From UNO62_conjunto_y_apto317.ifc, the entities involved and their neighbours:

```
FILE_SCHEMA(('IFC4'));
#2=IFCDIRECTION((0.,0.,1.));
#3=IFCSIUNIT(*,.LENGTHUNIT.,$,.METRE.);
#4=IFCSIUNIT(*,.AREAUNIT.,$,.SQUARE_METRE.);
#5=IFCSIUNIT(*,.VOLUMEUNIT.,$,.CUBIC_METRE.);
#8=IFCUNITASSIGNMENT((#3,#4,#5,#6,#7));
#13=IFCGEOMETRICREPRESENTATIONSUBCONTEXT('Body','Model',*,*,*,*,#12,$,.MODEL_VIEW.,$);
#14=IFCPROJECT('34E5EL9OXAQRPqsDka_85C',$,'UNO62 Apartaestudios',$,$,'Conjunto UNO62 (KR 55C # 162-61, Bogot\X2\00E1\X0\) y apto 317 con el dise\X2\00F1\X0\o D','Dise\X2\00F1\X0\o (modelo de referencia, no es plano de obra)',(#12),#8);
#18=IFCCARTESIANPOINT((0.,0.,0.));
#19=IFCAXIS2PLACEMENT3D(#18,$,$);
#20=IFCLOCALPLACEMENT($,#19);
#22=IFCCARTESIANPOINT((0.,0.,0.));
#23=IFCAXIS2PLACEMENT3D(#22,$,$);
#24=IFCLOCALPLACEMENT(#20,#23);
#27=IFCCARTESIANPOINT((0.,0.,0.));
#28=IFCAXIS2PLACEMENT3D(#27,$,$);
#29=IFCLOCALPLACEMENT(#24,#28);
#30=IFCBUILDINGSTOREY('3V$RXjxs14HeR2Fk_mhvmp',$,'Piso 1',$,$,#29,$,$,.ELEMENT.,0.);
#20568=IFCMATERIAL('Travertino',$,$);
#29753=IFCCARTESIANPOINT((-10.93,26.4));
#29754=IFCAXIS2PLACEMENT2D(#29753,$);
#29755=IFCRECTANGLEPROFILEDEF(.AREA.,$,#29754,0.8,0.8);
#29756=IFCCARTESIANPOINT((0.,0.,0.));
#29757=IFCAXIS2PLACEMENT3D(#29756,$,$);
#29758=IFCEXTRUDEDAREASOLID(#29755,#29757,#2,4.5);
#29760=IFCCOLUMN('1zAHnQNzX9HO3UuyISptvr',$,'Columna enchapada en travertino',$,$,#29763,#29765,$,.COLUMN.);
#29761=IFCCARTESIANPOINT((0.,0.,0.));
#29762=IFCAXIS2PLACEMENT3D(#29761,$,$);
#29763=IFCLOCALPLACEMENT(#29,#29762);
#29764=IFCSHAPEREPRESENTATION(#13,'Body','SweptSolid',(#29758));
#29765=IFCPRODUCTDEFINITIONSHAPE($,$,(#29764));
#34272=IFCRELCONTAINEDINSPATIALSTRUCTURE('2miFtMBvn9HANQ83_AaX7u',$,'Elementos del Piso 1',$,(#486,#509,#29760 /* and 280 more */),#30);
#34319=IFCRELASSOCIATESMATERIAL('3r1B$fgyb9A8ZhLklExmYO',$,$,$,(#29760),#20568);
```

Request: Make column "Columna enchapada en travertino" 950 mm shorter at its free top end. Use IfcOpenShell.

```python
import ifcopenshell
import ifcopenshell.util.representation
import ifcopenshell.util.unit

model = ifcopenshell.open("UNO62_conjunto_y_apto317.ifc")
unit_scale = ifcopenshell.util.unit.calculate_unit_scale(model)

member = model.by_guid("1zAHnQNzX9HO3UuyISptvr")
change = -0.95 / unit_scale

# The extrusion runs towards the end named, so only its depth changes.
body = ifcopenshell.util.representation.get_representation(member, "Model", "Body")
solid = body.Items[0]
old_length = solid.Depth
solid.Depth += change

print(f"length {old_length:g} -> {solid.Depth:g}")

model.write("UNO62_conjunto_y_apto317_rev.ifc")
```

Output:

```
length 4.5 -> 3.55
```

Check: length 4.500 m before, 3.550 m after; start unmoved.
